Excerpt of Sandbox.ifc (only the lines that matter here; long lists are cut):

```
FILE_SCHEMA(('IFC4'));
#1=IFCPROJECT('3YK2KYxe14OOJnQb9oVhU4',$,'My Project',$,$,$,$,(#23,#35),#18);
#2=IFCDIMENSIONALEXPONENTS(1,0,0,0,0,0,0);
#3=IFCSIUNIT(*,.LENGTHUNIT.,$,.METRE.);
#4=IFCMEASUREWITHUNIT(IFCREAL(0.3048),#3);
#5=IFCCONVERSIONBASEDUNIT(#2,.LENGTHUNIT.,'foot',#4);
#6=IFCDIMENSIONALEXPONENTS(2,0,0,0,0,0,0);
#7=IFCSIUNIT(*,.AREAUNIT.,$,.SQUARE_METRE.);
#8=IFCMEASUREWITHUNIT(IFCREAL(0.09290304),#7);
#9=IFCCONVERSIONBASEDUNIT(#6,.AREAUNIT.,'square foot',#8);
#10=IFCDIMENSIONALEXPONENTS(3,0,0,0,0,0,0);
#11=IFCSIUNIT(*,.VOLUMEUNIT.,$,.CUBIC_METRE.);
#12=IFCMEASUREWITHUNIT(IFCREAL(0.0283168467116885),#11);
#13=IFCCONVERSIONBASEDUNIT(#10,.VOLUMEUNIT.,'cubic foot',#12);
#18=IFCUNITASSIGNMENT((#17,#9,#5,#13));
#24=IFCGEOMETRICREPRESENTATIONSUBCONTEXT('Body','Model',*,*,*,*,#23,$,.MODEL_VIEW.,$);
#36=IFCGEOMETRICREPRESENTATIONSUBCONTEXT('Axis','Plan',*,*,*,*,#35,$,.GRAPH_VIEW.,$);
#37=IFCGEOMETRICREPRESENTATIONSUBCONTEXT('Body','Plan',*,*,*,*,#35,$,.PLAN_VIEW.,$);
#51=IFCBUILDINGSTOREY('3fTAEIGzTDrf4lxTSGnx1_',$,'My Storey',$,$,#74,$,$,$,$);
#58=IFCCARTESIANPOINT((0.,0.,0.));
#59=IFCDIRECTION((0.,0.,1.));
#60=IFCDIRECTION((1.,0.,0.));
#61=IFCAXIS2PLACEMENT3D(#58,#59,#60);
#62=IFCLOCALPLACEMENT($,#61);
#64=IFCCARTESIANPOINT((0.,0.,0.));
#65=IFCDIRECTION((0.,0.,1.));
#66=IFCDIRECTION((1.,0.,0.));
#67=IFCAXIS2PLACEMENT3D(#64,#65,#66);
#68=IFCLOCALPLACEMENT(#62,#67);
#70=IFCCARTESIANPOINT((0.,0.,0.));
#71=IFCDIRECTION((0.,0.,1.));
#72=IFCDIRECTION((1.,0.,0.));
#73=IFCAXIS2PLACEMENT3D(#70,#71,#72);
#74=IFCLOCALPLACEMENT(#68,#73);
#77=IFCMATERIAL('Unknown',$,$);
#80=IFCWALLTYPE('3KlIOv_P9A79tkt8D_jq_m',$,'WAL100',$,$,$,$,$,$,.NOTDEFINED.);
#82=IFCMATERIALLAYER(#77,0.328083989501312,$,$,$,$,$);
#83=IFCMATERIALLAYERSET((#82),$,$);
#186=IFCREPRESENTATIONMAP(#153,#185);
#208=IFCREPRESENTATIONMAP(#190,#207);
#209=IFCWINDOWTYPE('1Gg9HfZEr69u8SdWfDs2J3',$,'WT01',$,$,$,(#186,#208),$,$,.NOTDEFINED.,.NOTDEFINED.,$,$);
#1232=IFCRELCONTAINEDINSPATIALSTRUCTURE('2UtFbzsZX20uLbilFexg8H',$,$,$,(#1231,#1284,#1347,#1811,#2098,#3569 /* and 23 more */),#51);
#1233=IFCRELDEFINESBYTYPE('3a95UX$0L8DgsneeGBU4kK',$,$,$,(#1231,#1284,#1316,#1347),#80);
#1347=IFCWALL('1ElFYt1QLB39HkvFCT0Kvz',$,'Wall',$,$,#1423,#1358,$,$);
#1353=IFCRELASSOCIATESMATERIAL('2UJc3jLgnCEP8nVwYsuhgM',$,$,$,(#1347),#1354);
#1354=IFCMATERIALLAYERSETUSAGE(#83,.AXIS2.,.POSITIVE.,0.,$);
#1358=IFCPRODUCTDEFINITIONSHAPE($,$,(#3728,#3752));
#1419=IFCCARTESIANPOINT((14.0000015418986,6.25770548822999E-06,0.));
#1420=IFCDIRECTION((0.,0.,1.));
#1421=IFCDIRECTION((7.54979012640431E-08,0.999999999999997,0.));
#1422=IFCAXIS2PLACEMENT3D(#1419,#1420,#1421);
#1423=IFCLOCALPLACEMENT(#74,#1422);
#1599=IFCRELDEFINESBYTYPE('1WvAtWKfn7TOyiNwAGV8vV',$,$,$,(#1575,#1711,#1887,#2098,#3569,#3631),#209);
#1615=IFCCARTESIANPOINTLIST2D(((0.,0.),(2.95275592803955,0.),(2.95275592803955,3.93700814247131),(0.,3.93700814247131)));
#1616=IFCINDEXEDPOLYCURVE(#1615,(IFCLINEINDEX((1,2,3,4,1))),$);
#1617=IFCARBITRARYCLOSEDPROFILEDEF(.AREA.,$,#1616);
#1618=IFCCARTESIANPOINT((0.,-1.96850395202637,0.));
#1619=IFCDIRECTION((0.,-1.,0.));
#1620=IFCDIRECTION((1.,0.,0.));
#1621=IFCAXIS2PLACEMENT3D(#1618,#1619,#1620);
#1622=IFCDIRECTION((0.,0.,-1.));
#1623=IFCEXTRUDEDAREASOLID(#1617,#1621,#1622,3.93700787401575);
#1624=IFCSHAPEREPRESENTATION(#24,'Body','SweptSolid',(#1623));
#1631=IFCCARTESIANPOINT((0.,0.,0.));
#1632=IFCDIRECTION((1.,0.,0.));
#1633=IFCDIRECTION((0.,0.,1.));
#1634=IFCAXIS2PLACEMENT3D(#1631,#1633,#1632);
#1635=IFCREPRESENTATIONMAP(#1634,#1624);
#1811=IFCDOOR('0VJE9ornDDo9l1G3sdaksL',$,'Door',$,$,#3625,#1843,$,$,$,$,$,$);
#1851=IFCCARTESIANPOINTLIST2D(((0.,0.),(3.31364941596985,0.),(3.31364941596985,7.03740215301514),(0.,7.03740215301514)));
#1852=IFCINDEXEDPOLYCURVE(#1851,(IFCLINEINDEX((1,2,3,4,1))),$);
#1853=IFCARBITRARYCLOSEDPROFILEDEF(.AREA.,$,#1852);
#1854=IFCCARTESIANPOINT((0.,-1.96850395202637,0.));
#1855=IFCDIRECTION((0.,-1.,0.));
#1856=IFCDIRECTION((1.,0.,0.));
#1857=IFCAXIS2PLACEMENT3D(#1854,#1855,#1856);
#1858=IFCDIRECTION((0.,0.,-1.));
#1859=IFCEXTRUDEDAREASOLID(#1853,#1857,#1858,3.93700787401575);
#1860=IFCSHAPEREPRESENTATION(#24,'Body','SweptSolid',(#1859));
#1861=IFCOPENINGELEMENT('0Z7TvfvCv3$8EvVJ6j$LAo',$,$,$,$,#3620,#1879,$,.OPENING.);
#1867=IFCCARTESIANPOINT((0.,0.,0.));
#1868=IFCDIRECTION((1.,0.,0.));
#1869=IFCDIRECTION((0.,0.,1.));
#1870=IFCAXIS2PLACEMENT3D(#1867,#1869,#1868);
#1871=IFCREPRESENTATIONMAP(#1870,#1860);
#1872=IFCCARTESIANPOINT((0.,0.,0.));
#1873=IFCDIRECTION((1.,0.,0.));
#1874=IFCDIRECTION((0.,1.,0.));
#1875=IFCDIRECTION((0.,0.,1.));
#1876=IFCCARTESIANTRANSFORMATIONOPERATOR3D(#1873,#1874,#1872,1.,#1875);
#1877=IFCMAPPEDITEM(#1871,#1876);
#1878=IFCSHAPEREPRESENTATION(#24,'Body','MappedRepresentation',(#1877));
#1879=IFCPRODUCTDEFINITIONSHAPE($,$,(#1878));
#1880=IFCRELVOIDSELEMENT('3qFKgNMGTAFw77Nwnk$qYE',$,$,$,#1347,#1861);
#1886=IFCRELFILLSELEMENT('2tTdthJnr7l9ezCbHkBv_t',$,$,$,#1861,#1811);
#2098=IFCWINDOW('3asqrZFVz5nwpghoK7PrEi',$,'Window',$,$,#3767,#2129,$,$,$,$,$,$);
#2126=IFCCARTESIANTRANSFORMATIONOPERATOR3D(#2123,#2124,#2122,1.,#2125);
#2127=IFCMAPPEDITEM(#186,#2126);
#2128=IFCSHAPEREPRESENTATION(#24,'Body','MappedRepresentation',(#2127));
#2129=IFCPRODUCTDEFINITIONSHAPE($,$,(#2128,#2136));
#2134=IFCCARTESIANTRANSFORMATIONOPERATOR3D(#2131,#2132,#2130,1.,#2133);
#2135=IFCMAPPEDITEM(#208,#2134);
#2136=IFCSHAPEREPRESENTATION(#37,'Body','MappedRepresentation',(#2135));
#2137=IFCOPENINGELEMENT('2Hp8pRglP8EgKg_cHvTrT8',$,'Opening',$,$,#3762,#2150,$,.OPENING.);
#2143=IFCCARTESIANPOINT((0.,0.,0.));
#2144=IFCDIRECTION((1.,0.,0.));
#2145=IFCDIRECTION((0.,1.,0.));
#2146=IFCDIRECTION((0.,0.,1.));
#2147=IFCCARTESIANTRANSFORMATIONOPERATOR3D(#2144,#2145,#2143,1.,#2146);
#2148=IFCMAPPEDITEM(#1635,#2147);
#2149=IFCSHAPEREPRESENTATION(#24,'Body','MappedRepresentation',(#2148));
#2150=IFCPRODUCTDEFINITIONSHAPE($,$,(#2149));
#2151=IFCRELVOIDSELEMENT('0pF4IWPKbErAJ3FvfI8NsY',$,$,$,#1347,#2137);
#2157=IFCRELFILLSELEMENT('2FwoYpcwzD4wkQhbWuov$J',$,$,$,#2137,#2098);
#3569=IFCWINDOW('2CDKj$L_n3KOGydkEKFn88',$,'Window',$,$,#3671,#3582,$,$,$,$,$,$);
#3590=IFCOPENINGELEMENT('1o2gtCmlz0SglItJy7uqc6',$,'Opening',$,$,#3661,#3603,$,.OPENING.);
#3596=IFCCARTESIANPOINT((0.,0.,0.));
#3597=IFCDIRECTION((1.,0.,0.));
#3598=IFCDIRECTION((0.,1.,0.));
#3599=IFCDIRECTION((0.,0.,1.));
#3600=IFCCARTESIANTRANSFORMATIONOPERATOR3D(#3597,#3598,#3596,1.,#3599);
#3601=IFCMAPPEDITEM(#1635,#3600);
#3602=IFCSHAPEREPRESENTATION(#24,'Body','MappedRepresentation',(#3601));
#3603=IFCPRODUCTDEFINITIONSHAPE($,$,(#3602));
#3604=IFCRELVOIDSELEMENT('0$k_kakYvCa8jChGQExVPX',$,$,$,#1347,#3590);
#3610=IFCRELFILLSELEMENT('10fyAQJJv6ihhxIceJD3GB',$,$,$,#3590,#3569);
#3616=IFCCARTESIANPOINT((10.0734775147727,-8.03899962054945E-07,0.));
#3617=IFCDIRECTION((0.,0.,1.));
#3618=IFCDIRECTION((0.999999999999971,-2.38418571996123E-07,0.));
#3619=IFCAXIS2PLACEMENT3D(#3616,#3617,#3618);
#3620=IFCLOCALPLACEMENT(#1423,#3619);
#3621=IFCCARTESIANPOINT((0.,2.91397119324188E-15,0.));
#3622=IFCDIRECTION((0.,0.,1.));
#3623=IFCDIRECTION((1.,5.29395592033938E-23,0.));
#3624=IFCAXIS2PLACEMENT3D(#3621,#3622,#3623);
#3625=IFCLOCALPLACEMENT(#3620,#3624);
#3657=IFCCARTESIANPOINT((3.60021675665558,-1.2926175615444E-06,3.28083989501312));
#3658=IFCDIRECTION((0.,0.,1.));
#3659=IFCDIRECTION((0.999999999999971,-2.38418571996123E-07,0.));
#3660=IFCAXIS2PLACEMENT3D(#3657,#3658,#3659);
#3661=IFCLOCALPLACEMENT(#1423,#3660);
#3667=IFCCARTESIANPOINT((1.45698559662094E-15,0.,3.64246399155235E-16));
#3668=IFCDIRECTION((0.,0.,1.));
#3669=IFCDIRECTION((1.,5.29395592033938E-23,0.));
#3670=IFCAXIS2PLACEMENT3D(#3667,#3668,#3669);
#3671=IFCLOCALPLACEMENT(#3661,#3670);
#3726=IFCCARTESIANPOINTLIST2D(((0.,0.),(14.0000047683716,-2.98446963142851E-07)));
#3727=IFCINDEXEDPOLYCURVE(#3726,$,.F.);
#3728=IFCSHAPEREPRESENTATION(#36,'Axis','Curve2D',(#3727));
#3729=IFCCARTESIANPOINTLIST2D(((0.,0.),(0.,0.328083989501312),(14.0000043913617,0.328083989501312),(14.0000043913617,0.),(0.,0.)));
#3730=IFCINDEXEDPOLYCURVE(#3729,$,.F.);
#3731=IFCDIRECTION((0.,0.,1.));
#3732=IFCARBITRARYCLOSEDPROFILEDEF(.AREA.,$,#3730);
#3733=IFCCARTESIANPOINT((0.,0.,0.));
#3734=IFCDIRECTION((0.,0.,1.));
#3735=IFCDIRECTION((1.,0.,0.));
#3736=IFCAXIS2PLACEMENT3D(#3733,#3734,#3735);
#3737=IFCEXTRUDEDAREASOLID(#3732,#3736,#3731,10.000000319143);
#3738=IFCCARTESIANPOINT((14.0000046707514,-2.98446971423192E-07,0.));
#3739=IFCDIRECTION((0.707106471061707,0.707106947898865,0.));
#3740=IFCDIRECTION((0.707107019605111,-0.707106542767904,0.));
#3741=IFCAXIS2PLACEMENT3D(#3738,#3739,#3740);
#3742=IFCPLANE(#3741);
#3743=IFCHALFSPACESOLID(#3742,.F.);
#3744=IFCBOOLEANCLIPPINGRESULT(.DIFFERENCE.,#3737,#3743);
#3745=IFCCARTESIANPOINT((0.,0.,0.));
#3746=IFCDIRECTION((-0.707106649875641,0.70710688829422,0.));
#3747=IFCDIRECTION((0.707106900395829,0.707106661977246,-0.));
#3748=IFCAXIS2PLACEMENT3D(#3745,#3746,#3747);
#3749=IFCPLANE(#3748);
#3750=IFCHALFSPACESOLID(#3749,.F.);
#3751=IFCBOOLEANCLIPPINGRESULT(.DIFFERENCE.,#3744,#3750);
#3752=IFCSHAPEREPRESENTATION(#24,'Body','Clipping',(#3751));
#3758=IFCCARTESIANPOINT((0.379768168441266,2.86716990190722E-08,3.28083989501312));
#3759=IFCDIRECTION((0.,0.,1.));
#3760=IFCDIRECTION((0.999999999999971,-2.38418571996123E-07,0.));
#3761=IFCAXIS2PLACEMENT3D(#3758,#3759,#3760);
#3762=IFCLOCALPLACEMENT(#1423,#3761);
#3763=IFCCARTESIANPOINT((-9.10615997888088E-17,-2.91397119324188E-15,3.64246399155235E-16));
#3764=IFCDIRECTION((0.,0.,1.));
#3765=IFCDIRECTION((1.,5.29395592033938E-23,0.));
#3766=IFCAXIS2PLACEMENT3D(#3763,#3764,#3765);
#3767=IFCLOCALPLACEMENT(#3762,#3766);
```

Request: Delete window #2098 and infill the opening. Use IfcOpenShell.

```python
import ifcopenshell
import ifcopenshell.api.feature
import ifcopenshell.api.root
import ifcopenshell.geom
import ifcopenshell.util.shape

model = ifcopenshell.open("Sandbox.ifc")
settings = ifcopenshell.geom.settings()


def volume(element):
    """Net volume in cubic metres, openings subtracted."""
    shape = ifcopenshell.geom.create_shape(settings, element)
    return ifcopenshell.util.shape.get_volume(shape.geometry)


window = model.by_guid("3asqrZFVz5nwpghoK7PrEi")
opening = window.FillsVoids[0].RelatingOpeningElement
wall = opening.VoidsElements[0].RelatingBuildingElement
before = volume(wall)

ifcopenshell.api.root.remove_product(model, product=window)
ifcopenshell.api.feature.remove_feature(model, feature=opening)

after = volume(wall)

print(f"wall volume {before:.3f} -> {after:.3f} m3")

model.write("Sandbox_rev.ifc")
```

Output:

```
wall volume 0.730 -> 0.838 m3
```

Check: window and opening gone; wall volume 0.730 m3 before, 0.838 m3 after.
